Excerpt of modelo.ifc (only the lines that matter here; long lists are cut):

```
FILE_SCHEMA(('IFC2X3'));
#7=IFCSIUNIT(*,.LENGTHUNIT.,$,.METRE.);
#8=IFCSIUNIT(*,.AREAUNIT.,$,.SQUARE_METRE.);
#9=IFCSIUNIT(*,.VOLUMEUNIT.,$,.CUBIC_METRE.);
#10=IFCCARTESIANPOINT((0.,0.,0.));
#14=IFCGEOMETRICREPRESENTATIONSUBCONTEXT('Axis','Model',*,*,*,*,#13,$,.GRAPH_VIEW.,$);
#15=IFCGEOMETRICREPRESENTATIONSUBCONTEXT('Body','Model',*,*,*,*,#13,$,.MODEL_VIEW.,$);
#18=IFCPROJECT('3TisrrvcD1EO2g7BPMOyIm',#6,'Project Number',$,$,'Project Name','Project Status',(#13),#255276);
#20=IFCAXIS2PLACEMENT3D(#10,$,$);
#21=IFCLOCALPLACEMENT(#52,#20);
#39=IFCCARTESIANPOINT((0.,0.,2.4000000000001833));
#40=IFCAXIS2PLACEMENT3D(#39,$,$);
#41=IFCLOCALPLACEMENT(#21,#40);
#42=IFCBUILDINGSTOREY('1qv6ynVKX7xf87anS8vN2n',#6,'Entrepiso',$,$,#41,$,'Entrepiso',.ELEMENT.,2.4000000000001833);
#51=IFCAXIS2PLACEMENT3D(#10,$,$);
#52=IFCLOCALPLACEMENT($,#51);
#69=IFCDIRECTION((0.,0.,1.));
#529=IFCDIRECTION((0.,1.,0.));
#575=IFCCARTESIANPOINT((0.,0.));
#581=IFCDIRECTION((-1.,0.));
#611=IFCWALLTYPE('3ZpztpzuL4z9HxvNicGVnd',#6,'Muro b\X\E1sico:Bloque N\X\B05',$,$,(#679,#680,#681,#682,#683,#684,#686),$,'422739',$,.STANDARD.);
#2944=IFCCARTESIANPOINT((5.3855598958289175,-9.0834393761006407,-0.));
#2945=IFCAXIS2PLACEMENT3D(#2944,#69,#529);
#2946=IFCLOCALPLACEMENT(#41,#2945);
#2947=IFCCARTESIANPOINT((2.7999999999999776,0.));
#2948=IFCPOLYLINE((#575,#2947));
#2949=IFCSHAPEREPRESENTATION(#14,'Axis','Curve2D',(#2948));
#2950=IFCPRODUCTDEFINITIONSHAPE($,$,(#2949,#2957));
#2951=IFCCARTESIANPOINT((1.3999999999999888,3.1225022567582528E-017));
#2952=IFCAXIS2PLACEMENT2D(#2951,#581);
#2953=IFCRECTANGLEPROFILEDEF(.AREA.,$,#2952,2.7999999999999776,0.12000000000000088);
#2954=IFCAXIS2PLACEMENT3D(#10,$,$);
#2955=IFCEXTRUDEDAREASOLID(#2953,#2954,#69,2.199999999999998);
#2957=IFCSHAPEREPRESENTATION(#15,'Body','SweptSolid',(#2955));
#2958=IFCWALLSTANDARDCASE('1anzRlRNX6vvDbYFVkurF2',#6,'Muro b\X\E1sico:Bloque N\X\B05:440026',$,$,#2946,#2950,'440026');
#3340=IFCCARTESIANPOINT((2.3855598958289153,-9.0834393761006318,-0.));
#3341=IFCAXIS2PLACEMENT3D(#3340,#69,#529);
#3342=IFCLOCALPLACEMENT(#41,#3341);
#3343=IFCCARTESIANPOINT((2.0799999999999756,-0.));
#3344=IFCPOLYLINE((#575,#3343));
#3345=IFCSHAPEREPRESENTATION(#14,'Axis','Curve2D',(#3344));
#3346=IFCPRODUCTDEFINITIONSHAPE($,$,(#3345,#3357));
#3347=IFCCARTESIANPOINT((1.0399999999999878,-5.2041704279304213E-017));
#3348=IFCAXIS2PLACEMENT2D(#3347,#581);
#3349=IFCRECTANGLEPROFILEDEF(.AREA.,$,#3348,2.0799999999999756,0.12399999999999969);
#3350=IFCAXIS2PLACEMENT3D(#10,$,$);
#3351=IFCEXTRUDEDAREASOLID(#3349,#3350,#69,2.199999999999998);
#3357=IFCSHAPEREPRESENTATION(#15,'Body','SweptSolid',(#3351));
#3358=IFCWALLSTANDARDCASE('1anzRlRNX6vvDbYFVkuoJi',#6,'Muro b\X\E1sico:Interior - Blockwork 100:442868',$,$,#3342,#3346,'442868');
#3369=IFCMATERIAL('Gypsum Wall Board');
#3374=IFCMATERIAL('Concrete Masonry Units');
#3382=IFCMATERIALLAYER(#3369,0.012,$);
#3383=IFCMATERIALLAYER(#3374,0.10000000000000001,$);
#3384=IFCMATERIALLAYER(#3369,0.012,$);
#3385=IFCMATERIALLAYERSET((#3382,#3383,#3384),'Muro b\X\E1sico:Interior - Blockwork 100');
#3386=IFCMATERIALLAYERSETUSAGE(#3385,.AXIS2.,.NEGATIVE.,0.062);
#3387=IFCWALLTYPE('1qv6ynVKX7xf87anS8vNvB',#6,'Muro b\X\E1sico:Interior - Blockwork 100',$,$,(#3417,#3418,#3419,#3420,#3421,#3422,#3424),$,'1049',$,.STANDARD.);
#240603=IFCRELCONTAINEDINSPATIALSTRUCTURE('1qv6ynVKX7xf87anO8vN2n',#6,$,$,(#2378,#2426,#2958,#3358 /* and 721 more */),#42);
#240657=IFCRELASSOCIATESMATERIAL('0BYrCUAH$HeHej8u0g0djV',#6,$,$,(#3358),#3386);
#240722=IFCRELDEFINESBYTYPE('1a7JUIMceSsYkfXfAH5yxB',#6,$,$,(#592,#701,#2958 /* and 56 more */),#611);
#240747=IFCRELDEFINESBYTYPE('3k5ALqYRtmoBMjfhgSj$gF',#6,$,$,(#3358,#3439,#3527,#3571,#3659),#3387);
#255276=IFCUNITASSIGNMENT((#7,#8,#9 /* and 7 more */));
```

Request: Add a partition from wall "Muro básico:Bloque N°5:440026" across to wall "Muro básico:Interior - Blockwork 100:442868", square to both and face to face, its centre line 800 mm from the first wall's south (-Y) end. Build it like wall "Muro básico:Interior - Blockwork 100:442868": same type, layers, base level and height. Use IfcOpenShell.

```python
import numpy as np
import ifcopenshell
import ifcopenshell.api.geometry
import ifcopenshell.api.material
import ifcopenshell.api.pset
import ifcopenshell.api.root
import ifcopenshell.api.spatial
import ifcopenshell.api.type
import ifcopenshell.geom
import ifcopenshell.util.element
import ifcopenshell.util.placement
import ifcopenshell.util.representation
import ifcopenshell.util.shape
import ifcopenshell.util.unit

model = ifcopenshell.open("modelo.ifc")
unit_scale = ifcopenshell.util.unit.calculate_unit_scale(model)
settings = ifcopenshell.geom.settings()
settings.set("use-world-coords", True)

start_wall = model.by_id(2958)
end_wall = model.by_guid("1anzRlRNX6vvDbYFVkuoJi")
like = model.by_id(3358)
matrix = ifcopenshell.util.placement.get_local_placement(start_wall.ObjectPlacement)
matrix[:3, 3] *= unit_scale


def extent(element):
    """Bounding box in the first wall's axes, in metres."""
    shape = ifcopenshell.geom.create_shape(settings, element)
    points = (ifcopenshell.util.shape.get_vertices(shape.geometry) - matrix[:3, 3]) @ matrix[:3, :3]
    return points.min(axis=0), points.max(axis=0)


y_start = extent(start_wall)[1][1]
y_end = extent(end_wall)[0][1]
like_min, like_max = extent(like)
length, height = float(abs(y_end - y_start)), float(like_max[2] - like_min[2])
layer_set = ifcopenshell.util.element.get_material(like, should_skip_usage=True)
thickness = sum(layer.LayerThickness for layer in layer_set.MaterialLayers) * unit_scale

wall = ifcopenshell.api.root.create_entity(model, ifc_class="IfcWallStandardCase", name="New partition")
storey = ifcopenshell.util.element.get_container(like)
ifcopenshell.api.spatial.assign_container(model, products=[wall], relating_structure=storey)
ifcopenshell.api.type.assign_type(
    model, related_objects=[wall], relating_type=ifcopenshell.util.element.get_type(like), should_map_representations=False
)
rel = ifcopenshell.api.material.assign_material(
    model, products=[wall], type="IfcMaterialLayerSetUsage", material=layer_set
)
rel.RelatingMaterial.OffsetFromReferenceLine = -thickness / 2 / unit_scale
pset = ifcopenshell.api.pset.add_pset(model, product=wall, name="Pset_WallCommon")
ifcopenshell.api.pset.edit_pset(model, pset=pset, properties={"IsExternal": False, "LoadBearing": False})

# The axis runs down the middle of the wall.
axis = ifcopenshell.api.geometry.add_axis_representation(
    model, context=ifcopenshell.util.representation.get_context(model, "Model", "Axis"), axis=[(0.0, 0.0), (length, 0.0)]
)
body = ifcopenshell.api.geometry.add_wall_representation(
    model,
    context=ifcopenshell.util.representation.get_context(model, "Model", "Body", "MODEL_VIEW"),
    length=length,
    height=height,
    thickness=thickness,
    offset=-thickness / 2,
)
for representation in (axis, body):
    ifcopenshell.api.geometry.assign_representation(model, product=wall, representation=representation)

placement = matrix @ ifcopenshell.util.placement.rotation(90, "Z")
placement[:, 3] = matrix @ np.array([extent(start_wall)[0][0] + 0.8, y_start, like_min[2], 1.0])
ifcopenshell.api.geometry.edit_object_placement(model, product=wall, matrix=placement)

print(f"partition {length:.3f} m long, {height:.3f} m high, {thickness:.3f} m thick")

model.write("modelo_v2.ifc")
```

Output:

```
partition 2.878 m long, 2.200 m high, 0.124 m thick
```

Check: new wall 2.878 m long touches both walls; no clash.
